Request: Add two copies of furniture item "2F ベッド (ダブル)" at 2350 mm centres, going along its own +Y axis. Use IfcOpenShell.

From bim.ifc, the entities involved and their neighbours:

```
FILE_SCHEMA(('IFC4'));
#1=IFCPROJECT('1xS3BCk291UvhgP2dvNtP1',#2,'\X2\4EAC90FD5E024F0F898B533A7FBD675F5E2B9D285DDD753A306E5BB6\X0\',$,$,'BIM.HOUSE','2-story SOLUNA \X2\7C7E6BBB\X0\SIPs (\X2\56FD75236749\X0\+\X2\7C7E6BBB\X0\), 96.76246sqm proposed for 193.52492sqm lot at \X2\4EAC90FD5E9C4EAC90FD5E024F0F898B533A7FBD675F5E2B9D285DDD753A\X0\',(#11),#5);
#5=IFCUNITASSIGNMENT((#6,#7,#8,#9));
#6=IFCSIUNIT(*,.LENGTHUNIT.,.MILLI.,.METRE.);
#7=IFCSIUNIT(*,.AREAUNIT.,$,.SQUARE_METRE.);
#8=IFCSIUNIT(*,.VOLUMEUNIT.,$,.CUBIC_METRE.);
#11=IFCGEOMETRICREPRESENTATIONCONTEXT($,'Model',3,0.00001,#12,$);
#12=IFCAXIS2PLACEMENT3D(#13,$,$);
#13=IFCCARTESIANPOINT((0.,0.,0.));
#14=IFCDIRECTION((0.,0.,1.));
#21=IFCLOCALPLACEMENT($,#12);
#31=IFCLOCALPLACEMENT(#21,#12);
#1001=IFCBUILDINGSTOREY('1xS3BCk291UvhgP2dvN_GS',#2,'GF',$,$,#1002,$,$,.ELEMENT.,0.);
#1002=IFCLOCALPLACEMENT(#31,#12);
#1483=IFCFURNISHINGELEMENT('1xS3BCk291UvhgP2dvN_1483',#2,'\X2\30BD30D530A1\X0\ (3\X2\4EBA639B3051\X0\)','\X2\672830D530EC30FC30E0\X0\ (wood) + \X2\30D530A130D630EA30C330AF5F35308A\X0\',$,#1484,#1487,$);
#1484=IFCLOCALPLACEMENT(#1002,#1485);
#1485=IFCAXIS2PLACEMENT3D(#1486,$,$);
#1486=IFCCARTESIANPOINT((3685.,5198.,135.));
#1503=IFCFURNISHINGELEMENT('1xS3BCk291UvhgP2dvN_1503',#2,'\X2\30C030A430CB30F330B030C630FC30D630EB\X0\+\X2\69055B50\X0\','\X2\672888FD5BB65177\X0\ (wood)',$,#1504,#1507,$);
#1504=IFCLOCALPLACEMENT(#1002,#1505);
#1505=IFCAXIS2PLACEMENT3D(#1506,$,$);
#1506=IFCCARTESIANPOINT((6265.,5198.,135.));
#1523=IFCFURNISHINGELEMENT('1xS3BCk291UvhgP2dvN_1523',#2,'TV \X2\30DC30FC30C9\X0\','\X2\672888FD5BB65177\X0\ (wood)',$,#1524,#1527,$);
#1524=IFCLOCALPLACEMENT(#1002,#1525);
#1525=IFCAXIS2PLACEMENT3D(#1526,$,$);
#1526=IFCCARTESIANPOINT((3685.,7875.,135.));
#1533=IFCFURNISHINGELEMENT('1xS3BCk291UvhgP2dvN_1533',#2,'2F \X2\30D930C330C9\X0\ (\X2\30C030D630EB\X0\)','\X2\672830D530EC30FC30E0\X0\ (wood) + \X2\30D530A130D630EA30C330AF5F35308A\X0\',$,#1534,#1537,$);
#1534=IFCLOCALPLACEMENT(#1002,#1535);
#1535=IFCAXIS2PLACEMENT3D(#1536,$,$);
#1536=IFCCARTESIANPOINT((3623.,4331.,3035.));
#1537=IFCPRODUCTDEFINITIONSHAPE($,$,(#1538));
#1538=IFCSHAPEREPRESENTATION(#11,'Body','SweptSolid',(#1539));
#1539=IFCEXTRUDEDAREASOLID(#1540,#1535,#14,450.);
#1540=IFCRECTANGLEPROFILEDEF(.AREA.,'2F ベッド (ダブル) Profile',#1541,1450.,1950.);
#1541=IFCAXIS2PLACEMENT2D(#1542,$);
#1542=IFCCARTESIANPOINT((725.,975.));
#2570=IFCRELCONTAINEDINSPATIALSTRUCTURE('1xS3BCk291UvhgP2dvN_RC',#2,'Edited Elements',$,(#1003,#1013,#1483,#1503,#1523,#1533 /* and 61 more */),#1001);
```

```python
import ifcopenshell
import ifcopenshell.api.geometry
import ifcopenshell.api.root
import ifcopenshell.util.element
import ifcopenshell.util.placement
import ifcopenshell.util.unit

model = ifcopenshell.open("bim.ifc")
unit_scale = ifcopenshell.util.unit.calculate_unit_scale(model)


def reuse_history(source, copy):
    """copy_class also copies each property set's owner history, people and application; keep the originals."""
    for rel in copy.IsDefinedBy:
        if rel.is_a("IfcRelDefinesByProperties") and (history := rel.RelatingPropertyDefinition.OwnerHistory):
            rel.RelatingPropertyDefinition.OwnerHistory = source.OwnerHistory
            ifcopenshell.util.element.remove_deep2(model, history)


source = model.by_id(1533)
base = ifcopenshell.util.placement.get_local_placement(source.ObjectPlacement)
step = base[:3, 1] * 2.35 / unit_scale

for i in range(1, 3):
    copy = ifcopenshell.api.root.copy_class(model, product=source)
    copy.Representation = ifcopenshell.util.element.copy_deep(
        model, source.Representation, exclude=["IfcGeometricRepresentationContext", "IfcRepresentationMap"]
    )
    reuse_history(source, copy)
    matrix = base.copy()
    matrix[:3, 3] += i * step
    print("added at", matrix[:3, 3].round(3) + 0.0)
    ifcopenshell.api.geometry.edit_object_placement(model, product=copy, matrix=matrix, is_si=False)

model.write("bim_edited.ifc")
```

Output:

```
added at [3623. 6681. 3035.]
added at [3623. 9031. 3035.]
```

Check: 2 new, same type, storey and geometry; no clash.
